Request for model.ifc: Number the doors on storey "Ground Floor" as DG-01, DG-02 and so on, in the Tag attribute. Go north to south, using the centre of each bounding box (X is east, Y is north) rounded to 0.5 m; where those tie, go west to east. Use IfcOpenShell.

First a look at what the model holds.

```python
import ifcopenshell
import ifcopenshell.util.element
import ifcopenshell.util.placement

model = ifcopenshell.open("model.ifc")
print(model.schema)
storey = next(s for s in model.by_type("IfcBuildingStorey") if s.Name == "Ground Floor")
doors = [e for e in ifcopenshell.util.element.get_decomposition(storey) if e.is_a("IfcDoor")]
for e in sorted(doors, key=lambda e: e.id()):
    origin = ifcopenshell.util.placement.get_local_placement(e.ObjectPlacement)[:3, 3]
    print(e.id(), e.Tag, e.Name, origin.round(2) + 0.0, sep=" | ")
```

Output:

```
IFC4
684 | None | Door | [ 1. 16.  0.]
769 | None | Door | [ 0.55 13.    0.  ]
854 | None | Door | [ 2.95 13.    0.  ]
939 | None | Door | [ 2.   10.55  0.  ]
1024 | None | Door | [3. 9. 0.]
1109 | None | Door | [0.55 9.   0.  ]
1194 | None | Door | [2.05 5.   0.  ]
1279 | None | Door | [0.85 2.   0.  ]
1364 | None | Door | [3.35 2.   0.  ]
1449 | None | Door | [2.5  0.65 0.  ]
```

```python
import ifcopenshell
import ifcopenshell.geom
import ifcopenshell.util.element
import ifcopenshell.util.shape

model = ifcopenshell.open("model.ifc")
settings = ifcopenshell.geom.settings()
settings.set("use-world-coords", True)


def centre(element):
    shape = ifcopenshell.geom.create_shape(settings, element)
    return ifcopenshell.util.shape.get_bbox_centroid(shape.geometry)


storey = next(s for s in model.by_type("IfcBuildingStorey") if s.Name == "Ground Floor")
doors = [e for e in ifcopenshell.util.element.get_decomposition(storey) if e.is_a("IfcDoor")]

# Insertion points can sit at a corner or the storey origin, so sort by the geometry (in metres).
centres = {e: centre(e) for e in doors}
doors.sort(key=lambda e: (-round(centres[e][1] / 0.5), centres[e][0]))

for i, e in enumerate(doors, start=1):
    number = f"DG-{i:02d}"
    e.Tag = number
    print(e.id(), number)

model.write("model_rev.ifc")
```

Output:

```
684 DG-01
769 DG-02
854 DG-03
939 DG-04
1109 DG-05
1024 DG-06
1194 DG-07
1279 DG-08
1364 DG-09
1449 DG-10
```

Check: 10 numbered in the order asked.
